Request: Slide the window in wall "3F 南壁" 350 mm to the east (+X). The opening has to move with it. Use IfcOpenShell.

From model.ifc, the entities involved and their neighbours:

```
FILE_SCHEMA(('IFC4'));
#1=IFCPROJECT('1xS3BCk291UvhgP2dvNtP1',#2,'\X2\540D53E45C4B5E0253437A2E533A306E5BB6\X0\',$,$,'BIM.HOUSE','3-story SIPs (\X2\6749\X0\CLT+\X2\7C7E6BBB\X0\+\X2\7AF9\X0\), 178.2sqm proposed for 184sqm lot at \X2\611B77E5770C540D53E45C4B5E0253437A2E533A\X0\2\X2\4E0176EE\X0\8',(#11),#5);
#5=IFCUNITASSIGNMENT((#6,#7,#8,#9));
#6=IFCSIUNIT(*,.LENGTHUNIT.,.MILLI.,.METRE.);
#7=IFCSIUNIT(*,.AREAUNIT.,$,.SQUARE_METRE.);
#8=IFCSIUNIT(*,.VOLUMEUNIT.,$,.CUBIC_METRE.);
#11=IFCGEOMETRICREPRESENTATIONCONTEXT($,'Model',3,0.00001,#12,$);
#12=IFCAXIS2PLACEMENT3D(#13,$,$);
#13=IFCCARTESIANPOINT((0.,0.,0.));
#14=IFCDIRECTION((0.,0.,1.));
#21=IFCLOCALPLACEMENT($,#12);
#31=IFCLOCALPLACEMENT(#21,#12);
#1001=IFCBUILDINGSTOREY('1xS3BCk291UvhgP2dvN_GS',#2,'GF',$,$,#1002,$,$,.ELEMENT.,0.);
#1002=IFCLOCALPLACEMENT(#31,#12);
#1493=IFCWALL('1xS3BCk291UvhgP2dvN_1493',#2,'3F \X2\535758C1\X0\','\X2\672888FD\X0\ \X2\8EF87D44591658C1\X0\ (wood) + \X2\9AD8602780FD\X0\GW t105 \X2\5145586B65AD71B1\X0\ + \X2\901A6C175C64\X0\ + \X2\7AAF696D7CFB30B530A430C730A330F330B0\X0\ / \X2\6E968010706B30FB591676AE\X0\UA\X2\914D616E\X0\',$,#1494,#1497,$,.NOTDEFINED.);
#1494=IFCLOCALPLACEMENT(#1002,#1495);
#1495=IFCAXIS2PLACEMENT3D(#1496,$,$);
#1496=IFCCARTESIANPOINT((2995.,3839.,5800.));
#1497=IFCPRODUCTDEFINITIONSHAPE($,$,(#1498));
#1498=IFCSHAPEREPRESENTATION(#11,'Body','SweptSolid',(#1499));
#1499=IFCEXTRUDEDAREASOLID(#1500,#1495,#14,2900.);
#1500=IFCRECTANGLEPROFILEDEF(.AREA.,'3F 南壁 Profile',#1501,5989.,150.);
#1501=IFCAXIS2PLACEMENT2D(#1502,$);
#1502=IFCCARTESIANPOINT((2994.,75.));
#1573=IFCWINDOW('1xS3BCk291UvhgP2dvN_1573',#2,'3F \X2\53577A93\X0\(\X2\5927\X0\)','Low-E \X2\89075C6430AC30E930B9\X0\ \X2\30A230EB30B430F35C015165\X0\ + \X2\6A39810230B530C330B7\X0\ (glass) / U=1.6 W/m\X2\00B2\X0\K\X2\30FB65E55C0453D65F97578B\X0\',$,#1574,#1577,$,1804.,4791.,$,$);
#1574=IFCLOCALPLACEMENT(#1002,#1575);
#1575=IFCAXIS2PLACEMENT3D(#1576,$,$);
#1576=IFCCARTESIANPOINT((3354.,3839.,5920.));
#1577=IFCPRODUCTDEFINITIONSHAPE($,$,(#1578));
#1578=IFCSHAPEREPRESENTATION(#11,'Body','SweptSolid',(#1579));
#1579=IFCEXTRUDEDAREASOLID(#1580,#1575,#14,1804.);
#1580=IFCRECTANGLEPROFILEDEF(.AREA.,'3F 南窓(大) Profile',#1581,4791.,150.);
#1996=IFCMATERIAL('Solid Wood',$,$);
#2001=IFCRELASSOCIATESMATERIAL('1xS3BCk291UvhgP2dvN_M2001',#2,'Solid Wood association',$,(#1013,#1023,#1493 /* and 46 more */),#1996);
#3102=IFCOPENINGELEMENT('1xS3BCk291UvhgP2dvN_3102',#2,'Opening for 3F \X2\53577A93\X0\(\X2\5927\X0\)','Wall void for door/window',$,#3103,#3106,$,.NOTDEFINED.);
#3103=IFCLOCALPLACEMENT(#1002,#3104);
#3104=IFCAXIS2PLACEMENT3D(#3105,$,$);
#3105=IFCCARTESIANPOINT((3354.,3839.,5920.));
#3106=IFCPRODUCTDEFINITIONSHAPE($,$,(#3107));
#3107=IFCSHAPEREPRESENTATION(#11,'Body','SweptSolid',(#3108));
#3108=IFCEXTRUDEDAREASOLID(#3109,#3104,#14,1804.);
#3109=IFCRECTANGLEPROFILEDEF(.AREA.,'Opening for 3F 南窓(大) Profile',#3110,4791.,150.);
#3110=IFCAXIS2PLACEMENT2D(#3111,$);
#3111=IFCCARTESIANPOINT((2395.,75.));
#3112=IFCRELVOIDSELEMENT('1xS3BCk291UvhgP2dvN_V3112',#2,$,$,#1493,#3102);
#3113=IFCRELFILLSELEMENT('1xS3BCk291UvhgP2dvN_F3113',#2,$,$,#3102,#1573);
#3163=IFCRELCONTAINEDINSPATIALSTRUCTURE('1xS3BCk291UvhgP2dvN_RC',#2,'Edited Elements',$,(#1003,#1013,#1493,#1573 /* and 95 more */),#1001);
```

```python
import ifcopenshell
import ifcopenshell.api.geometry
import ifcopenshell.util.placement

model = ifcopenshell.open("model.ifc")

window = model.by_guid("1xS3BCk291UvhgP2dvN_1573")
opening = window.FillsVoids[0].RelatingOpeningElement
wall = opening.VoidsElements[0].RelatingBuildingElement

wall_matrix = ifcopenshell.util.placement.get_local_placement(wall.ObjectPlacement)
shift = wall_matrix[:3, 0] * 350.0
before = ifcopenshell.util.placement.get_local_placement(window.ObjectPlacement)[:3, 3].copy()

# The window is not placed relative to its opening, so move both.
for product in (opening, window):
    matrix = ifcopenshell.util.placement.get_local_placement(product.ObjectPlacement)
    matrix[:3, 3] += shift
    ifcopenshell.api.geometry.edit_object_placement(model, product=product, matrix=matrix, is_si=False)

after = ifcopenshell.util.placement.get_local_placement(window.ObjectPlacement)[:3, 3]
print("window moved by", (after - before).round(3) + 0.0)

model.write("model_updated.ifc")
```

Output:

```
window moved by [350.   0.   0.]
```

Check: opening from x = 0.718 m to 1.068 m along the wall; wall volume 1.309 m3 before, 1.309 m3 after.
